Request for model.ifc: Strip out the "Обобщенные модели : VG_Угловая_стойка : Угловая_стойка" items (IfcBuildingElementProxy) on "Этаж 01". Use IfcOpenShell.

First a look at what the model holds.

```python
import ifcopenshell
import ifcopenshell.util.element

model = ifcopenshell.open("model.ifc")
print(model.schema)
storey = next(s for s in model.by_type("IfcBuildingStorey") if s.Name == "Этаж 01")
proxies = [e for e in ifcopenshell.util.element.get_decomposition(storey) if e.is_a("IfcBuildingElementProxy")]
seen = {}
for e in proxies:
    element_type = ifcopenshell.util.element.get_type(e)
    name = element_type.Name if element_type not in (None, e) else None
    seen[name] = seen.get(name, 0) + 1
for name, count in sorted(seen.items(), key=str):
    print(count, "x", name)
```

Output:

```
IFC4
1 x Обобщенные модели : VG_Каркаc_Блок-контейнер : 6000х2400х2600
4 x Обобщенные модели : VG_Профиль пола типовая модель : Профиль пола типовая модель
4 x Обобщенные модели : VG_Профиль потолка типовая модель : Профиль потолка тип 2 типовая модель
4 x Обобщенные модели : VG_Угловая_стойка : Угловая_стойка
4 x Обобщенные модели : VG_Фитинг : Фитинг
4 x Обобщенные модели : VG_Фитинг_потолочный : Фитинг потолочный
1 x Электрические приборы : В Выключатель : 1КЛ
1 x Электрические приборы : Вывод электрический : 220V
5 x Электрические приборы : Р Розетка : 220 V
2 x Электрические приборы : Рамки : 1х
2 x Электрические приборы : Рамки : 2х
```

```python
import ifcopenshell
import ifcopenshell.api.root
import ifcopenshell.util.element

model = ifcopenshell.open("model.ifc")

storey = next(s for s in model.by_type("IfcBuildingStorey") if s.Name == "Этаж 01")
proxies = [e for e in ifcopenshell.util.element.get_decomposition(storey) if e.is_a("IfcBuildingElementProxy")]
targets = [e for e in proxies if (t := ifcopenshell.util.element.get_type(e)) not in (None, e) and t.Name == "Обобщенные модели : VG_Угловая_стойка : Угловая_стойка"]

for e in targets:
    ifcopenshell.api.root.remove_product(model, product=e)
print(len(targets), "removed")

model.write("model-out.ifc")
```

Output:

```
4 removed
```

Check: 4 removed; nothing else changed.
